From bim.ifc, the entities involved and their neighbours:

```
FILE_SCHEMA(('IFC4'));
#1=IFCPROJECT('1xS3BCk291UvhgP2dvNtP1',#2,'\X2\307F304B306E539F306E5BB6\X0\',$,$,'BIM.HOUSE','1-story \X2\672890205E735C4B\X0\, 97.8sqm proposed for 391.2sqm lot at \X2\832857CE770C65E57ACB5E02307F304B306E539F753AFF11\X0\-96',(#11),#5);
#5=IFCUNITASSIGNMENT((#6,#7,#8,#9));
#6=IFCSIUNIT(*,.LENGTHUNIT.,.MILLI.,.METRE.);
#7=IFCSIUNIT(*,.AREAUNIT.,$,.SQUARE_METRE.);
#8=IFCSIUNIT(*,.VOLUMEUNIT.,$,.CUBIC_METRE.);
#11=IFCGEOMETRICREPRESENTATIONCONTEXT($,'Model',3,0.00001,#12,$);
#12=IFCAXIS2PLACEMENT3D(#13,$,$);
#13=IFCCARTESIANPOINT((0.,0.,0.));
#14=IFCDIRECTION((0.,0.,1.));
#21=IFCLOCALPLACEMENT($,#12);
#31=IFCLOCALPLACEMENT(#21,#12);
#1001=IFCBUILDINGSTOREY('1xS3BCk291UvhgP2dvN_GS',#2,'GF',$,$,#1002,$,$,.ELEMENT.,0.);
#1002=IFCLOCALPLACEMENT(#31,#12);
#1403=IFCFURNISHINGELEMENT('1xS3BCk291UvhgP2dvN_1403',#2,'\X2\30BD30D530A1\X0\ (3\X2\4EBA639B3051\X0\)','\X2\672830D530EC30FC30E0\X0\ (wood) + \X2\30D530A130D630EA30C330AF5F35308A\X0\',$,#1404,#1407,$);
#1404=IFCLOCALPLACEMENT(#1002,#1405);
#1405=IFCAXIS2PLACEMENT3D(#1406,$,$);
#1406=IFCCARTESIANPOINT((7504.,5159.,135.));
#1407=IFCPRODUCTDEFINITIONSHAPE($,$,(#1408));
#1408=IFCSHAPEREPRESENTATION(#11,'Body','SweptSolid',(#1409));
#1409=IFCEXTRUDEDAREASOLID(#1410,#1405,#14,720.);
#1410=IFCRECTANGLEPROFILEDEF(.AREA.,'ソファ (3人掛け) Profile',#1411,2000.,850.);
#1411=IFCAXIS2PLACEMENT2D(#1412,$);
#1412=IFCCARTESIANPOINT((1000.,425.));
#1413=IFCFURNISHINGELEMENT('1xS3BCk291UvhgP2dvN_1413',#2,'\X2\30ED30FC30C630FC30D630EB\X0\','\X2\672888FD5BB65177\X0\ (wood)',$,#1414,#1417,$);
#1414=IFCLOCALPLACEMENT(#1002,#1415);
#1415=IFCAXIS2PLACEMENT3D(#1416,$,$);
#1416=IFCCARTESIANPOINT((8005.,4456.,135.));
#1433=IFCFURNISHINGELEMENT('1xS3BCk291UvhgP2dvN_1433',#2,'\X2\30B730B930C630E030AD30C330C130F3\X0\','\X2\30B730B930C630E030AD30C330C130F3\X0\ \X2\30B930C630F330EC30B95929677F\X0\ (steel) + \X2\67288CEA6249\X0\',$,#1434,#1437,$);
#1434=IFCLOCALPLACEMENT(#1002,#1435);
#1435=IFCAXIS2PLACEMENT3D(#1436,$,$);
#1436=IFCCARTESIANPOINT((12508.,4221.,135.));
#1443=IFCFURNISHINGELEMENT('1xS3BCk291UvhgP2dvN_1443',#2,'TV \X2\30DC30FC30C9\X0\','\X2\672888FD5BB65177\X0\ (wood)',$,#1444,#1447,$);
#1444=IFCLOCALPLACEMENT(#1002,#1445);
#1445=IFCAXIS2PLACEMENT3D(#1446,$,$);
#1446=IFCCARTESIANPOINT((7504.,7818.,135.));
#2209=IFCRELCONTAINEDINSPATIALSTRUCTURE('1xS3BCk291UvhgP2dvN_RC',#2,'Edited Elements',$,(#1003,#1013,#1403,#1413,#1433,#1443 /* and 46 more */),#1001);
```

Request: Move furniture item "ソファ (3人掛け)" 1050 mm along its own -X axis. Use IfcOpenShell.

```python
import ifcopenshell
import ifcopenshell.api.geometry
import ifcopenshell.util.placement

model = ifcopenshell.open("bim.ifc")

item = model.by_id(1403)
matrix = ifcopenshell.util.placement.get_local_placement(item.ObjectPlacement)
matrix[:3, 3] -= matrix[:3, 0] * 1050.0
ifcopenshell.api.geometry.edit_object_placement(model, product=item, matrix=matrix, is_si=False)

print(ifcopenshell.util.placement.get_local_placement(item.ObjectPlacement).round(3) + 0.0)

model.write("bim_v2.ifc")
```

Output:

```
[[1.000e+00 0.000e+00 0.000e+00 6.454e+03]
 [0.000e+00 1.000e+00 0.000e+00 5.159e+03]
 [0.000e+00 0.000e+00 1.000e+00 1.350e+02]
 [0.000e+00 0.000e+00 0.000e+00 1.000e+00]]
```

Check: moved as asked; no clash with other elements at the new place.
